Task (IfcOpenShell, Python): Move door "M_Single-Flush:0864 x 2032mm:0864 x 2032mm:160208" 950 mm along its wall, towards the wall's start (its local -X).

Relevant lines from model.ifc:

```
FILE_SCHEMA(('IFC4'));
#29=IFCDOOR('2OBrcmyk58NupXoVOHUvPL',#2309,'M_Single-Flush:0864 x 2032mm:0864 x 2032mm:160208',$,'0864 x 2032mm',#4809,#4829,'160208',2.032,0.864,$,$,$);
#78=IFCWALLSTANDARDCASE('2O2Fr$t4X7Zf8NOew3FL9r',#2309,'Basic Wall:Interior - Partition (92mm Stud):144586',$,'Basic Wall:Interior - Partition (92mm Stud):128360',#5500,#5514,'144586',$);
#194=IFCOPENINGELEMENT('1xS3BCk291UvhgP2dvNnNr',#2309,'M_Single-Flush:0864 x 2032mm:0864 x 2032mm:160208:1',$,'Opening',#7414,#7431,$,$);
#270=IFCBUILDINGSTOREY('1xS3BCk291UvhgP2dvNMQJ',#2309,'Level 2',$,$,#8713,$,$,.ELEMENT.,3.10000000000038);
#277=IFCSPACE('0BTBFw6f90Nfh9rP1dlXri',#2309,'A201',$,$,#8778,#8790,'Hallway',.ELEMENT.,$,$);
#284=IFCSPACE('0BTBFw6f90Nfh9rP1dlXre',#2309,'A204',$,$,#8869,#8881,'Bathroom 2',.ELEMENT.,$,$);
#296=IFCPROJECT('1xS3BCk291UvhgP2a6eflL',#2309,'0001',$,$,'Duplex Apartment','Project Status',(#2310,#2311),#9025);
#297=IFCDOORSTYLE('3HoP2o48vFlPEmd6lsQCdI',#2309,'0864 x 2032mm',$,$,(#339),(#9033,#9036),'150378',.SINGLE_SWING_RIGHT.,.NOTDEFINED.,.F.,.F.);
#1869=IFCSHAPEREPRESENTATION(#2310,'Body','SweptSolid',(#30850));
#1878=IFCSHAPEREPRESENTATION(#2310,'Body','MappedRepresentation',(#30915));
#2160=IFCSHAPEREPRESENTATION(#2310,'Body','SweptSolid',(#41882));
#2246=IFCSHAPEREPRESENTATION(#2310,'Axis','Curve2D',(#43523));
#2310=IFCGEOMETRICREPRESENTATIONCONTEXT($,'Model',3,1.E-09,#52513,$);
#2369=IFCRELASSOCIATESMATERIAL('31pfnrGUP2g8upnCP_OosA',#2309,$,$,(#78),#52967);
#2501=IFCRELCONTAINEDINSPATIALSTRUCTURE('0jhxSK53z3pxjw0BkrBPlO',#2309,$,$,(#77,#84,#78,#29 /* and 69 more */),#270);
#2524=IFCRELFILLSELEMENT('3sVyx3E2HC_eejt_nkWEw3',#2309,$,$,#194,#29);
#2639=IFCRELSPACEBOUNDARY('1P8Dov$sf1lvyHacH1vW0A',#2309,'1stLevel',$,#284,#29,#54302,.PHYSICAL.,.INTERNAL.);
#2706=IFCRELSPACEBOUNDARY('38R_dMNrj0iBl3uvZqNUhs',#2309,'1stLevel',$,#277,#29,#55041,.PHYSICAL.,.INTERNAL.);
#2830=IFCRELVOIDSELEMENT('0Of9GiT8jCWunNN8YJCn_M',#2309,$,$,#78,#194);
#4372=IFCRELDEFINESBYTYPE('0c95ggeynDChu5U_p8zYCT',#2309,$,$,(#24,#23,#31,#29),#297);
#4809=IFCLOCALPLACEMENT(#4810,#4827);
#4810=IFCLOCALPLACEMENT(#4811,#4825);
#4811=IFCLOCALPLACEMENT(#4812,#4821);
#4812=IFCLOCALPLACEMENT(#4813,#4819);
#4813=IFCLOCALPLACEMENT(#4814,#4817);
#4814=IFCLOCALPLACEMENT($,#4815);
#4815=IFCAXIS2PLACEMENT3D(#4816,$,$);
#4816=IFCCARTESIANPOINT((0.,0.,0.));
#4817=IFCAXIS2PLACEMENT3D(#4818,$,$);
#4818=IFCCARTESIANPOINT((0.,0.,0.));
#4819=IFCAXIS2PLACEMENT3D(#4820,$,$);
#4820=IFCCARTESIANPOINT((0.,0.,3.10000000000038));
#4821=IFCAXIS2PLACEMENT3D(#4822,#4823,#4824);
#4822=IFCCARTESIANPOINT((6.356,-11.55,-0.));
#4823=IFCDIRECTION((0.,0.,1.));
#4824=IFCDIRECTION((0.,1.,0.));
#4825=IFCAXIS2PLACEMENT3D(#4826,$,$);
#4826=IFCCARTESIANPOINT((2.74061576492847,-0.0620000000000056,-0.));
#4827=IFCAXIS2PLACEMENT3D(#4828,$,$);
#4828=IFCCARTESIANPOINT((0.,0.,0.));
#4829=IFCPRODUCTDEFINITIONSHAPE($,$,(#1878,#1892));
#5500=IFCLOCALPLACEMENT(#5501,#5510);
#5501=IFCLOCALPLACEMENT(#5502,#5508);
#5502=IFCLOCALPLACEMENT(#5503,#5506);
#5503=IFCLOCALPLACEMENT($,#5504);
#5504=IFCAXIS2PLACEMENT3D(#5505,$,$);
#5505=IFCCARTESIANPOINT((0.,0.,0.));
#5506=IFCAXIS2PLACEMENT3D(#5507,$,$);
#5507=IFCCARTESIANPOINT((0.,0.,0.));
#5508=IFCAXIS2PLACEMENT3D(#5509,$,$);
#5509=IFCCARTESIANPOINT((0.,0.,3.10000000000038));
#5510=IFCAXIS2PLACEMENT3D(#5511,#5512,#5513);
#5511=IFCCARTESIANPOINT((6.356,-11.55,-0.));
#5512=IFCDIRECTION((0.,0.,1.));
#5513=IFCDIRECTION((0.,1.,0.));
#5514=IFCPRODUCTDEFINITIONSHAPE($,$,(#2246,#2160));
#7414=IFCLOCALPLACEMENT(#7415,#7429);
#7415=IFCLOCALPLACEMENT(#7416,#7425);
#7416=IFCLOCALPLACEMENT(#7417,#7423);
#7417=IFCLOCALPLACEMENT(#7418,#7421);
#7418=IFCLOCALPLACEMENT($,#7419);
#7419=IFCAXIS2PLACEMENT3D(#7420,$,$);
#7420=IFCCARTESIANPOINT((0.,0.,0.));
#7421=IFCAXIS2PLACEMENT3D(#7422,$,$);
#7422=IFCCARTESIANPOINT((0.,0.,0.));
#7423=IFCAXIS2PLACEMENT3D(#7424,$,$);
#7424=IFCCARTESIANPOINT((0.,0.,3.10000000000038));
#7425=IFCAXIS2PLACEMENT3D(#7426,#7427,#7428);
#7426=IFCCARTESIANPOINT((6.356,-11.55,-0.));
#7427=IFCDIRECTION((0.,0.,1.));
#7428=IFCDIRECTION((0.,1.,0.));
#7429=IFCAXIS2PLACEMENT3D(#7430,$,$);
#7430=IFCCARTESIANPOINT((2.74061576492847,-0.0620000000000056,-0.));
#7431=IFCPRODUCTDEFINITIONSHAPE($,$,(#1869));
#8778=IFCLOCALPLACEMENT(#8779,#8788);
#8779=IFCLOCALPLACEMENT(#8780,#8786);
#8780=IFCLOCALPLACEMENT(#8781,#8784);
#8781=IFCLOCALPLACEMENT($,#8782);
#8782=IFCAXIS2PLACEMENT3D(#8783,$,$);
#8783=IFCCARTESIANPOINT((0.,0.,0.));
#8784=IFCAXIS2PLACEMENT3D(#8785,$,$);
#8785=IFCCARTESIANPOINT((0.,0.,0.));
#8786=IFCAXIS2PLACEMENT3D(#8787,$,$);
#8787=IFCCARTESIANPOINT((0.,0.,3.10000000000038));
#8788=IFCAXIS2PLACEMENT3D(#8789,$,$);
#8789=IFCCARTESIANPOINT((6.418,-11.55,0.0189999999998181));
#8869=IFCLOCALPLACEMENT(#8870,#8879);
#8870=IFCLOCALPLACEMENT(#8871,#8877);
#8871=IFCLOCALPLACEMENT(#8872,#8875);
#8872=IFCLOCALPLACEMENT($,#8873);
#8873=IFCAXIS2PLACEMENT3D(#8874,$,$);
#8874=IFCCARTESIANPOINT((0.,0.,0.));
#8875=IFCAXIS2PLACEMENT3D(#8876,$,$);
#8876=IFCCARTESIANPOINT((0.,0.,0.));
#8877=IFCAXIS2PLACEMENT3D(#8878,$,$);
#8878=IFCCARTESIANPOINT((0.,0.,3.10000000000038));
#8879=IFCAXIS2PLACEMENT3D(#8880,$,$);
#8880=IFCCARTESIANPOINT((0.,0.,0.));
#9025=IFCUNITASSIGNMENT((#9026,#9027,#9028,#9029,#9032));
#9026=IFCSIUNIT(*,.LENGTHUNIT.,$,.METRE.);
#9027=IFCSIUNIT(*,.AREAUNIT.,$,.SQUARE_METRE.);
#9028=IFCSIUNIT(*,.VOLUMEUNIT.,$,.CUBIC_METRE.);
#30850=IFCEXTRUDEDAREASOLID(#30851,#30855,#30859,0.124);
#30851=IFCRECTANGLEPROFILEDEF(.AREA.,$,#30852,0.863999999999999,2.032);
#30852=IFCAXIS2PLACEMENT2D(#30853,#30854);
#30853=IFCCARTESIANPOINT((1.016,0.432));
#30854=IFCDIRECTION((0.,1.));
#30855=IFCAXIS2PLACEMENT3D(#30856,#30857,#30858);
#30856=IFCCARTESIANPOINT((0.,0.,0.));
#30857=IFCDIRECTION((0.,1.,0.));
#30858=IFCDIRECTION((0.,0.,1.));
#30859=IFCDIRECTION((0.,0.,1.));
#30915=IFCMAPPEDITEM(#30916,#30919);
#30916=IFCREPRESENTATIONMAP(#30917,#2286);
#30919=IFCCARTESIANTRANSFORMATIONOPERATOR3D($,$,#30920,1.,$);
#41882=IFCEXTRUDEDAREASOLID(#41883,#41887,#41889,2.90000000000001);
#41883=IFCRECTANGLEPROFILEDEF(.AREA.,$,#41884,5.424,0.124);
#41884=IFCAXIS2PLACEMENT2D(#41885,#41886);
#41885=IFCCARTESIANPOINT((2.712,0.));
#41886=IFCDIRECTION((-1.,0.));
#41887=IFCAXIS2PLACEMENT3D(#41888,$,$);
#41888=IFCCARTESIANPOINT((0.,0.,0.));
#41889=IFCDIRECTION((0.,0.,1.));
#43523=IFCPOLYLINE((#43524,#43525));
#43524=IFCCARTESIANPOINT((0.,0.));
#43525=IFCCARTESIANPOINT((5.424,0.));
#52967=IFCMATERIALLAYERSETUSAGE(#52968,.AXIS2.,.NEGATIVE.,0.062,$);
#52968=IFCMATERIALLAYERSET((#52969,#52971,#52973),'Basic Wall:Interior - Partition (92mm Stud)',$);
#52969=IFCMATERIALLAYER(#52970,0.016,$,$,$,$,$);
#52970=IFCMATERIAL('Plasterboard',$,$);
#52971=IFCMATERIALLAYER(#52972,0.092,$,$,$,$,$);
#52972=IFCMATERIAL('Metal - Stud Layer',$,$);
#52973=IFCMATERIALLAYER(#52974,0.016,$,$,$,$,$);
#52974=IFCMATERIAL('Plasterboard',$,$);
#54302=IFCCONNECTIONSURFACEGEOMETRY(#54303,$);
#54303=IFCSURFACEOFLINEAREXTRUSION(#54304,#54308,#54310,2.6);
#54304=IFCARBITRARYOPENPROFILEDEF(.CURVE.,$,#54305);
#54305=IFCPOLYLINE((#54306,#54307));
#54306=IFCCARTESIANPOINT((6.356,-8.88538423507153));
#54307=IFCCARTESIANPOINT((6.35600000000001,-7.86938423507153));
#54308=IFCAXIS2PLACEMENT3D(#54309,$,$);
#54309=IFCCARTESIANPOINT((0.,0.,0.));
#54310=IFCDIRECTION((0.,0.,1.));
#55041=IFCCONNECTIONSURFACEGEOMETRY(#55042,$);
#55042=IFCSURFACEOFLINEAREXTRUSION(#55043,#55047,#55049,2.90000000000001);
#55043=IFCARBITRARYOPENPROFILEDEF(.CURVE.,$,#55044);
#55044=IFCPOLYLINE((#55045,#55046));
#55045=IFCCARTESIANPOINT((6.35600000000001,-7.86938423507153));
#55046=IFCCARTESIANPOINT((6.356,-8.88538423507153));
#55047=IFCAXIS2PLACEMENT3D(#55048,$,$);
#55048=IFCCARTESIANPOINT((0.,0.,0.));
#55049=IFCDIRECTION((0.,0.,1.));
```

```python
import numpy as np
import ifcopenshell
import ifcopenshell.api.geometry
import ifcopenshell.util.placement

model = ifcopenshell.open("model.ifc")

door = model.by_guid("2OBrcmyk58NupXoVOHUvPL")
opening = door.FillsVoids[0].RelatingOpeningElement
wall = opening.VoidsElements[0].RelatingBuildingElement

wall_matrix = ifcopenshell.util.placement.get_local_placement(wall.ObjectPlacement)
shift = wall_matrix[:3, 0] * -0.95
before = ifcopenshell.util.placement.get_local_placement(door.ObjectPlacement)[:3, 3].copy()

# The door is not placed relative to its opening, so move both.
for product in (opening, door):
    matrix = ifcopenshell.util.placement.get_local_placement(product.ObjectPlacement)
    matrix[:3, 3] += shift
    ifcopenshell.api.geometry.edit_object_placement(model, product=product, matrix=matrix, is_si=False)

# Space boundary surfaces are stored in each space's coordinates; move them too.
for rel in door.ProvidesBoundaries:
    if not rel.ConnectionGeometry:
        continue
    surface = rel.ConnectionGeometry.SurfaceOnRelatingElement
    space_matrix = ifcopenshell.util.placement.get_local_placement(rel.RelatingSpace.ObjectPlacement)
    point = np.array(surface.Position.Location.Coordinates) + space_matrix[:3, :3].T @ shift
    surface.Position = model.createIfcAxis2Placement3D(
        model.createIfcCartesianPoint(point.tolist()), surface.Position.Axis, surface.Position.RefDirection
    )

after = ifcopenshell.util.placement.get_local_placement(door.ObjectPlacement)[:3, 3]
print("door moved by", (after - before).round(3) + 0.0)

model.write("model-out.ifc")
```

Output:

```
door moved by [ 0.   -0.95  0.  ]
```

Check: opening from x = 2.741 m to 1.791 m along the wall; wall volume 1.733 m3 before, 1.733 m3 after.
